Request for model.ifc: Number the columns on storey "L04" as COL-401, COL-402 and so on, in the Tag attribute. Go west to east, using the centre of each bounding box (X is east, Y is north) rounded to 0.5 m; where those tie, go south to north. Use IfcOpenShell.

First a look at what the model holds.

```python
import ifcopenshell
import ifcopenshell.util.element
import ifcopenshell.util.placement

model = ifcopenshell.open("model.ifc")
print(model.schema)
storey = next(s for s in model.by_type("IfcBuildingStorey") if s.Name == "L04")
columns = [e for e in ifcopenshell.util.element.get_decomposition(storey) if e.is_a("IfcColumn")]
for e in sorted(columns, key=lambda e: e.id()):
    origin = ifcopenshell.util.placement.get_local_placement(e.ObjectPlacement)[:3, 3]
    print(e.id(), e.Tag, e.Name, origin.round(2) + 0.0, sep=" | ")
```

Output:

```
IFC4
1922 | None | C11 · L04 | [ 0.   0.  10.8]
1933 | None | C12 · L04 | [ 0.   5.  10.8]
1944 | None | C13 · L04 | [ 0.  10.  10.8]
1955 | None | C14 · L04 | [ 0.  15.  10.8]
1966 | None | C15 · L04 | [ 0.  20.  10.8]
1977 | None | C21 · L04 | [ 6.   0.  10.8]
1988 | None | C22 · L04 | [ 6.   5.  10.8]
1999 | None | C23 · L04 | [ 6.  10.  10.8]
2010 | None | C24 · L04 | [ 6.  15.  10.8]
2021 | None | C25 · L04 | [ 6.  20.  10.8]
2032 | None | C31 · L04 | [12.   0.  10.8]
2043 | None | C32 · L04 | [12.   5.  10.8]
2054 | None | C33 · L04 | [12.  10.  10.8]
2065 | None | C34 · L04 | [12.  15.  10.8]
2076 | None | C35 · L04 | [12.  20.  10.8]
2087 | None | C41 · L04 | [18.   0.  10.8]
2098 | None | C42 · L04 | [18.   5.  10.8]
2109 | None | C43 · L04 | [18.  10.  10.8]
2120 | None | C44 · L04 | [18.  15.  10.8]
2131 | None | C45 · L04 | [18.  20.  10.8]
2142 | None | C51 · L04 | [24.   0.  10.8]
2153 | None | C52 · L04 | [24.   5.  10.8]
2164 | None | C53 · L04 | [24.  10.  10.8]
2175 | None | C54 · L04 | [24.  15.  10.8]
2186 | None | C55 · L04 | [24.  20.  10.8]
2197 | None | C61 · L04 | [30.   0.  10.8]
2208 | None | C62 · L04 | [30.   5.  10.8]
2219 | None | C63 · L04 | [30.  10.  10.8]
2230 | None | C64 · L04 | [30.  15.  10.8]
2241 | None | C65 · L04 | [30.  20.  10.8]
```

```python
import ifcopenshell
import ifcopenshell.geom
import ifcopenshell.util.element
import ifcopenshell.util.shape

model = ifcopenshell.open("model.ifc")
settings = ifcopenshell.geom.settings()
settings.set("use-world-coords", True)


def centre(element):
    shape = ifcopenshell.geom.create_shape(settings, element)
    return ifcopenshell.util.shape.get_bbox_centroid(shape.geometry)


storey = next(s for s in model.by_type("IfcBuildingStorey") if s.Name == "L04")
columns = [e for e in ifcopenshell.util.element.get_decomposition(storey) if e.is_a("IfcColumn")]

# Insertion points can sit at a corner or the storey origin, so sort by the geometry (in metres).
centres = {e: centre(e) for e in columns}
columns.sort(key=lambda e: (round(centres[e][0] / 0.5), centres[e][1]))

for i, e in enumerate(columns, start=1):
    number = f"COL-4{i:02d}"
    e.Tag = number
    print(e.id(), number)

model.write("model-out.ifc")
```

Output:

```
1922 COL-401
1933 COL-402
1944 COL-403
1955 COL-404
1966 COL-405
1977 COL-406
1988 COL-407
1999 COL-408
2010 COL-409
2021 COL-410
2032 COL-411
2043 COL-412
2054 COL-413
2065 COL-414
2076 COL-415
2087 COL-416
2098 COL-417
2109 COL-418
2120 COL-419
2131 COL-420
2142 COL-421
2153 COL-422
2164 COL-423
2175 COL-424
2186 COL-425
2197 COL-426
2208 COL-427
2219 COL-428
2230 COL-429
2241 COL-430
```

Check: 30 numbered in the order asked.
